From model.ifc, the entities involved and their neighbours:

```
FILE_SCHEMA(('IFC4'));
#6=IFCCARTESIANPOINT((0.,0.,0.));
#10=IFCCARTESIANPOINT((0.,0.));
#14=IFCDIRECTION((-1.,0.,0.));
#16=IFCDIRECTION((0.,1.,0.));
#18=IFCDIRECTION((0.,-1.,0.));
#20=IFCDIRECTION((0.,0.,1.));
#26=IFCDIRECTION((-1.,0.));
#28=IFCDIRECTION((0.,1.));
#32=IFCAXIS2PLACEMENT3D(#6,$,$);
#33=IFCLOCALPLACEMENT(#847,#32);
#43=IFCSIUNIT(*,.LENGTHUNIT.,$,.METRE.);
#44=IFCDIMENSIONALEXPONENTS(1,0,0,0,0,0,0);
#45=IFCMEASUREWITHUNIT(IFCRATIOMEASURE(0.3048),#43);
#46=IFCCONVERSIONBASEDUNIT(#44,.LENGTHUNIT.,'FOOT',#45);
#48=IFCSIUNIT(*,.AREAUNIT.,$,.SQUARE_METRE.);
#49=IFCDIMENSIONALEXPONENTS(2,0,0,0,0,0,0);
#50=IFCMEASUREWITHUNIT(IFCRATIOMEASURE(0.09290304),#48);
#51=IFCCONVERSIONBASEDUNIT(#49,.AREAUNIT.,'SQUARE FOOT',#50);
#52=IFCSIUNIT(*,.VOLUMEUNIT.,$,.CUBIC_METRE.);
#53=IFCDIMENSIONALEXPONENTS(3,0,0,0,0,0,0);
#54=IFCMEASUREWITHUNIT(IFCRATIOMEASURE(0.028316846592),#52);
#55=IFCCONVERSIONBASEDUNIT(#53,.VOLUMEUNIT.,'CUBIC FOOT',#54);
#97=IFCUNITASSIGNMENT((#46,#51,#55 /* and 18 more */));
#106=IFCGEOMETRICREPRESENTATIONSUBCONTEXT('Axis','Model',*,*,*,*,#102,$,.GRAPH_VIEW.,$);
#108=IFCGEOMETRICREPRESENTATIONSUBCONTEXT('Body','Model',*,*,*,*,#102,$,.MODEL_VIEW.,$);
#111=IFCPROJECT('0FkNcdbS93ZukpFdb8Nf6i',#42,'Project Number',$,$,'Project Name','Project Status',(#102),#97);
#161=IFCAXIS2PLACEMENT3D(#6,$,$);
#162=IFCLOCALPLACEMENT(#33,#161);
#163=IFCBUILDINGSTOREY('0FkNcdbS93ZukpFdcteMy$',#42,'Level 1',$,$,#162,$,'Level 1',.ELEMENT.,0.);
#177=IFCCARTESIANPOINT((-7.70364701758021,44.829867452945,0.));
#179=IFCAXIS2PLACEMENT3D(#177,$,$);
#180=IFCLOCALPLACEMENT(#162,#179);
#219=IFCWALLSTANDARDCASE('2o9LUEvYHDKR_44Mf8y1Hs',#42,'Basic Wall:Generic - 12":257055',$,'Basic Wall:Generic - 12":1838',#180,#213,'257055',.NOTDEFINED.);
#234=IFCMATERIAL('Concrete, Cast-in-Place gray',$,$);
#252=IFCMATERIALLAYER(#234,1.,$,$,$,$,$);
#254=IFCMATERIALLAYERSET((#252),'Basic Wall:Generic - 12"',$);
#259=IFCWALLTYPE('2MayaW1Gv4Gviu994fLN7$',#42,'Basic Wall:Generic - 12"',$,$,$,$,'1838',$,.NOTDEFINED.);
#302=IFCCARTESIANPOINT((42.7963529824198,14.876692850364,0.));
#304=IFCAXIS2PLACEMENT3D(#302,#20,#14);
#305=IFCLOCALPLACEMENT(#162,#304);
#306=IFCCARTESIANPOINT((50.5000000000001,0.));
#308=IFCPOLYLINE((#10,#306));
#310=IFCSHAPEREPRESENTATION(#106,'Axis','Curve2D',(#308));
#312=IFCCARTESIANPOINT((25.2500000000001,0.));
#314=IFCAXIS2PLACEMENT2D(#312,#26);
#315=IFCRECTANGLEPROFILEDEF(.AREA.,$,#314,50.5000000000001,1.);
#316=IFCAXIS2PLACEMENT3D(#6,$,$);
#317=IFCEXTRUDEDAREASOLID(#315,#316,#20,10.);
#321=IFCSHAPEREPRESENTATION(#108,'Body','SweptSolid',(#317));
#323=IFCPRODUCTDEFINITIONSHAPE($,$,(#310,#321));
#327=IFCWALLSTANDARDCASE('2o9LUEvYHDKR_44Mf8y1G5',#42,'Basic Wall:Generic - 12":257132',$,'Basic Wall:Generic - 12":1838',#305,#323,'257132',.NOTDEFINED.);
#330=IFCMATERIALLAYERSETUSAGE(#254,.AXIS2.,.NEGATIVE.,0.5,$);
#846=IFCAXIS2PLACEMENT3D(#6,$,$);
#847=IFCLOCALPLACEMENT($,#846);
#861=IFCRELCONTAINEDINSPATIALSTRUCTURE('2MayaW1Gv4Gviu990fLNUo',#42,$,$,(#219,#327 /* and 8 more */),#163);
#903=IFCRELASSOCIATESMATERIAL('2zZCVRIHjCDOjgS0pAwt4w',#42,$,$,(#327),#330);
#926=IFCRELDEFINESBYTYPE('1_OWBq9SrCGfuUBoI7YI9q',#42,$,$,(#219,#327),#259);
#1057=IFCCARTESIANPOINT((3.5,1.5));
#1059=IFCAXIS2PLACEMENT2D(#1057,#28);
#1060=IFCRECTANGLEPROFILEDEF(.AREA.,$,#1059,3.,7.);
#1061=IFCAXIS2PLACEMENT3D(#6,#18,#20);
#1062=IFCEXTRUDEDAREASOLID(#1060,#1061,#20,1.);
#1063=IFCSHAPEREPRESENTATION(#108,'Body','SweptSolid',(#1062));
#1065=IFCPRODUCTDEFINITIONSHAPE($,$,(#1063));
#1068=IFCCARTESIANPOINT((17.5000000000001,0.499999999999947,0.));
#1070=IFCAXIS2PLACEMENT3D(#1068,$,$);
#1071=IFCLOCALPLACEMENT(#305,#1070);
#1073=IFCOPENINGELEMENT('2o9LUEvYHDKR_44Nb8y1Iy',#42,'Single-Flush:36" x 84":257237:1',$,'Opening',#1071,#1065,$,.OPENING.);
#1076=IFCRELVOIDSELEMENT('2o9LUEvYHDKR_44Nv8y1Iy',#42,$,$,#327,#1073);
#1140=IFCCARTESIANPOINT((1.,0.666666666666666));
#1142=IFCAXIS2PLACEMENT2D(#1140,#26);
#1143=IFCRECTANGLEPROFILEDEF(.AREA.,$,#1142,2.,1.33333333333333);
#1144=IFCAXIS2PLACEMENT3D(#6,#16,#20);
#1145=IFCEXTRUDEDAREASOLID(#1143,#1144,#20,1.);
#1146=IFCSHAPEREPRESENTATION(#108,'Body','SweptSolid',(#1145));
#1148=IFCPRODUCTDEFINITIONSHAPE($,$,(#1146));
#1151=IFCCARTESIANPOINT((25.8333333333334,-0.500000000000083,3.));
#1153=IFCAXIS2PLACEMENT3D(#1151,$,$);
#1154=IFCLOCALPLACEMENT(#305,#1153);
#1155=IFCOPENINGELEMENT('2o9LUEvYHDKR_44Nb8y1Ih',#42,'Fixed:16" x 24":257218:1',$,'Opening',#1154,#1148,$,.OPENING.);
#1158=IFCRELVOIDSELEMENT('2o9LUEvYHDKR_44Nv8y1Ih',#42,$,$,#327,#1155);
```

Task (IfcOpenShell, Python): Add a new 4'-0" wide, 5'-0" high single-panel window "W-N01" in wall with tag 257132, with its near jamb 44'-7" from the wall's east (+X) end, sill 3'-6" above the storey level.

```python
import numpy as np
import ifcopenshell
import ifcopenshell.api.feature
import ifcopenshell.api.geometry
import ifcopenshell.api.root
import ifcopenshell.api.spatial
import ifcopenshell.geom
import ifcopenshell.util.element
import ifcopenshell.util.placement
import ifcopenshell.util.representation
import ifcopenshell.util.shape
import ifcopenshell.util.unit

model = ifcopenshell.open("model.ifc")
unit_scale = ifcopenshell.util.unit.calculate_unit_scale(model)
settings = ifcopenshell.geom.settings()


def volume(element):
    """Net volume in cubic metres, openings subtracted."""
    shape = ifcopenshell.geom.create_shape(settings, element)
    return ifcopenshell.util.shape.get_volume(shape.geometry)


wall = model.by_guid("2o9LUEvYHDKR_44Mf8y1G5")
storey = ifcopenshell.util.element.get_container(wall, ifc_class="IfcBuildingStorey")
context = ifcopenshell.util.representation.get_context(model, "Model", "Body", "MODEL_VIEW")
before = volume(wall)

width, height, from_end, sill = 1.2192, 1.524, 13.589, 1.0668  # metres

# The wall runs along its own X axis, and the end named is its -X end.
wall_shape = ifcopenshell.geom.create_shape(settings, wall)
x, y, z = ifcopenshell.util.shape.get_vertices(wall_shape.geometry).T
start = x.min() + from_end
face, thickness = float(y.min()), float(y.max() - y.min())
wall_matrix = ifcopenshell.util.placement.get_local_placement(wall.ObjectPlacement)
level = ifcopenshell.util.placement.get_local_placement(storey.ObjectPlacement)[2, 3]


def in_wall(x, y):
    """Placement at x, y metres in the wall's axes, at sill height."""
    matrix = wall_matrix.copy()
    matrix[:, 3] = wall_matrix @ np.array([x / unit_scale, y / unit_scale, 0.0, 1.0])
    matrix[2, 3] = level + sill / unit_scale
    return matrix


# Opening: a box that overshoots both wall faces by 50 mm.
opening = ifcopenshell.api.root.create_entity(model, ifc_class="IfcOpeningElement", predefined_type="OPENING")
box = ifcopenshell.api.geometry.add_wall_representation(
    model, context=context, length=width, height=height, thickness=thickness + 0.1
)
ifcopenshell.api.geometry.assign_representation(model, product=opening, representation=box)
ifcopenshell.api.geometry.edit_object_placement(model, product=opening, matrix=in_wall(start, face - 0.05), is_si=False)
ifcopenshell.api.feature.add_feature(model, feature=opening, element=wall)

window = ifcopenshell.api.root.create_entity(model, ifc_class="IfcWindow", name="W-N01", predefined_type="WINDOW")
window.OverallWidth, window.OverallHeight = width / unit_scale, height / unit_scale
window.PartitioningType = "SINGLE_PANEL"
body = ifcopenshell.api.geometry.add_window_representation(
    model,
    context=context,
    overall_width=window.OverallWidth,
    overall_height=window.OverallHeight,
    partition_type="SINGLE_PANEL",
)
ifcopenshell.api.geometry.assign_representation(model, product=window, representation=body)
ifcopenshell.api.spatial.assign_container(model, products=[window], relating_structure=storey)
ifcopenshell.api.feature.add_filling(model, opening=opening, element=window)

# Centre the window in the wall's thickness.
ifcopenshell.api.geometry.edit_object_placement(model, product=window, matrix=in_wall(start, face), is_si=False)
window_shape = ifcopenshell.geom.create_shape(settings, window)
depth = ifcopenshell.util.shape.get_vertices(window_shape.geometry)[:, 1]
offset = face + thickness / 2 - (depth.min() + depth.max()) / 2
ifcopenshell.api.geometry.edit_object_placement(model, product=window, matrix=in_wall(start, offset), is_si=False)

after = volume(wall)

print(f"wall volume {before:.3f} -> {after:.3f} m3")

model.write("model_updated.ifc")
```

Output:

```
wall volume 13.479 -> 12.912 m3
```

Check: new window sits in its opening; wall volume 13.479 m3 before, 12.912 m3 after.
